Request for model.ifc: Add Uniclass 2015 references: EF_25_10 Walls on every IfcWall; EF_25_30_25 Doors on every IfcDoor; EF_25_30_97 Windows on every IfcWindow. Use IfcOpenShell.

First a look at what the model holds.

```python
import ifcopenshell

model = ifcopenshell.open("model.ifc")
print(model.schema)
print("classifications:", [c.Name for c in model.by_type("IfcClassification")])
for ifc_class in ("IfcDoor", "IfcRoof", "IfcStair", "IfcWall", "IfcWindow"):
    print(ifc_class, len(model.by_type(ifc_class)))
```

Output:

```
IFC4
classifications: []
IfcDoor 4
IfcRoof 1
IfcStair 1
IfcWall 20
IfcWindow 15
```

```python
import ifcopenshell
import ifcopenshell.api.classification

model = ifcopenshell.open("model.ifc")

system = ifcopenshell.api.classification.add_classification(model, classification="Uniclass 2015")

codes = {
    "IfcWall": ("EF_25_10", "Walls"),
    "IfcDoor": ("EF_25_30_25", "Doors"),
    "IfcWindow": ("EF_25_30_97", "Windows"),
}
for ifc_class, (code, name) in codes.items():
    products = model.by_type(ifc_class)
    ifcopenshell.api.classification.add_reference(
        model, products=products, classification=system, identification=code, name=name
    )
    print(code, len(products))

model.write("model_updated.ifc")
```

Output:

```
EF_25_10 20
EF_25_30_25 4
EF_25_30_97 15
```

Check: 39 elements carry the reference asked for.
